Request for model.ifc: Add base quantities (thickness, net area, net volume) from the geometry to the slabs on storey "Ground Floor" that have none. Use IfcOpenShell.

First a look at what the model holds.

```python
import ifcopenshell
import ifcopenshell.util.element
import ifcopenshell.util.unit

model = ifcopenshell.open("model.ifc")
print(model.schema)
for unit_type in ("LENGTHUNIT", "AREAUNIT", "VOLUMEUNIT"):
    print(unit_type, ifcopenshell.util.unit.calculate_unit_scale(model, unit_type))
storey = next(s for s in model.by_type("IfcBuildingStorey") if s.Name == "Ground Floor")
slabs = [e for e in ifcopenshell.util.element.get_decomposition(storey) if e.is_a("IfcSlab")]
for e in sorted(slabs, key=lambda e: e.id()):
    print(e.id(), e.is_a(), e.Name, list(ifcopenshell.util.element.get_psets(e, qtos_only=True)), sep=" | ")
```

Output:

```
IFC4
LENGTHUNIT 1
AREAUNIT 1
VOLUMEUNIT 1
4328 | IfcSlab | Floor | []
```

```python
import ifcopenshell
import ifcopenshell.api.pset
import ifcopenshell.geom
import ifcopenshell.util.element
import ifcopenshell.util.shape
import ifcopenshell.util.unit

model = ifcopenshell.open("model.ifc")
unit_scale = ifcopenshell.util.unit.calculate_unit_scale(model)
area_scale = ifcopenshell.util.unit.calculate_unit_scale(model, "AREAUNIT")
volume_scale = ifcopenshell.util.unit.calculate_unit_scale(model, "VOLUMEUNIT")
settings = ifcopenshell.geom.settings()

storey = next(s for s in model.by_type("IfcBuildingStorey") if s.Name == "Ground Floor")
slabs = [e for e in ifcopenshell.util.element.get_decomposition(storey) if e.is_a("IfcSlab")]

for e in sorted(slabs, key=lambda e: e.id()):
    if ifcopenshell.util.element.get_psets(e, qtos_only=True, should_inherit=False):
        continue
    # Geometry comes back in metres, in the element's own axes.
    shape = ifcopenshell.geom.create_shape(settings, e)
    values = {
        "Width": ifcopenshell.util.shape.get_z(shape.geometry) / unit_scale,
        "NetArea": ifcopenshell.util.shape.get_footprint_area(shape.geometry) / area_scale,
        "NetVolume": ifcopenshell.util.shape.get_volume(shape.geometry) / volume_scale,
    }
    qto = ifcopenshell.api.pset.add_qto(model, product=e, name="Qto_SlabBaseQuantities")
    ifcopenshell.api.pset.edit_qto(model, qto=qto, properties=values)
    print(e.id(), {k: round(v, 3) for k, v in values.items()})

model.write("model_v2.ifc")
```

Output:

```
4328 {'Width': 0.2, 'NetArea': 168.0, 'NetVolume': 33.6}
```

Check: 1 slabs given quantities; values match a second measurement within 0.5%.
